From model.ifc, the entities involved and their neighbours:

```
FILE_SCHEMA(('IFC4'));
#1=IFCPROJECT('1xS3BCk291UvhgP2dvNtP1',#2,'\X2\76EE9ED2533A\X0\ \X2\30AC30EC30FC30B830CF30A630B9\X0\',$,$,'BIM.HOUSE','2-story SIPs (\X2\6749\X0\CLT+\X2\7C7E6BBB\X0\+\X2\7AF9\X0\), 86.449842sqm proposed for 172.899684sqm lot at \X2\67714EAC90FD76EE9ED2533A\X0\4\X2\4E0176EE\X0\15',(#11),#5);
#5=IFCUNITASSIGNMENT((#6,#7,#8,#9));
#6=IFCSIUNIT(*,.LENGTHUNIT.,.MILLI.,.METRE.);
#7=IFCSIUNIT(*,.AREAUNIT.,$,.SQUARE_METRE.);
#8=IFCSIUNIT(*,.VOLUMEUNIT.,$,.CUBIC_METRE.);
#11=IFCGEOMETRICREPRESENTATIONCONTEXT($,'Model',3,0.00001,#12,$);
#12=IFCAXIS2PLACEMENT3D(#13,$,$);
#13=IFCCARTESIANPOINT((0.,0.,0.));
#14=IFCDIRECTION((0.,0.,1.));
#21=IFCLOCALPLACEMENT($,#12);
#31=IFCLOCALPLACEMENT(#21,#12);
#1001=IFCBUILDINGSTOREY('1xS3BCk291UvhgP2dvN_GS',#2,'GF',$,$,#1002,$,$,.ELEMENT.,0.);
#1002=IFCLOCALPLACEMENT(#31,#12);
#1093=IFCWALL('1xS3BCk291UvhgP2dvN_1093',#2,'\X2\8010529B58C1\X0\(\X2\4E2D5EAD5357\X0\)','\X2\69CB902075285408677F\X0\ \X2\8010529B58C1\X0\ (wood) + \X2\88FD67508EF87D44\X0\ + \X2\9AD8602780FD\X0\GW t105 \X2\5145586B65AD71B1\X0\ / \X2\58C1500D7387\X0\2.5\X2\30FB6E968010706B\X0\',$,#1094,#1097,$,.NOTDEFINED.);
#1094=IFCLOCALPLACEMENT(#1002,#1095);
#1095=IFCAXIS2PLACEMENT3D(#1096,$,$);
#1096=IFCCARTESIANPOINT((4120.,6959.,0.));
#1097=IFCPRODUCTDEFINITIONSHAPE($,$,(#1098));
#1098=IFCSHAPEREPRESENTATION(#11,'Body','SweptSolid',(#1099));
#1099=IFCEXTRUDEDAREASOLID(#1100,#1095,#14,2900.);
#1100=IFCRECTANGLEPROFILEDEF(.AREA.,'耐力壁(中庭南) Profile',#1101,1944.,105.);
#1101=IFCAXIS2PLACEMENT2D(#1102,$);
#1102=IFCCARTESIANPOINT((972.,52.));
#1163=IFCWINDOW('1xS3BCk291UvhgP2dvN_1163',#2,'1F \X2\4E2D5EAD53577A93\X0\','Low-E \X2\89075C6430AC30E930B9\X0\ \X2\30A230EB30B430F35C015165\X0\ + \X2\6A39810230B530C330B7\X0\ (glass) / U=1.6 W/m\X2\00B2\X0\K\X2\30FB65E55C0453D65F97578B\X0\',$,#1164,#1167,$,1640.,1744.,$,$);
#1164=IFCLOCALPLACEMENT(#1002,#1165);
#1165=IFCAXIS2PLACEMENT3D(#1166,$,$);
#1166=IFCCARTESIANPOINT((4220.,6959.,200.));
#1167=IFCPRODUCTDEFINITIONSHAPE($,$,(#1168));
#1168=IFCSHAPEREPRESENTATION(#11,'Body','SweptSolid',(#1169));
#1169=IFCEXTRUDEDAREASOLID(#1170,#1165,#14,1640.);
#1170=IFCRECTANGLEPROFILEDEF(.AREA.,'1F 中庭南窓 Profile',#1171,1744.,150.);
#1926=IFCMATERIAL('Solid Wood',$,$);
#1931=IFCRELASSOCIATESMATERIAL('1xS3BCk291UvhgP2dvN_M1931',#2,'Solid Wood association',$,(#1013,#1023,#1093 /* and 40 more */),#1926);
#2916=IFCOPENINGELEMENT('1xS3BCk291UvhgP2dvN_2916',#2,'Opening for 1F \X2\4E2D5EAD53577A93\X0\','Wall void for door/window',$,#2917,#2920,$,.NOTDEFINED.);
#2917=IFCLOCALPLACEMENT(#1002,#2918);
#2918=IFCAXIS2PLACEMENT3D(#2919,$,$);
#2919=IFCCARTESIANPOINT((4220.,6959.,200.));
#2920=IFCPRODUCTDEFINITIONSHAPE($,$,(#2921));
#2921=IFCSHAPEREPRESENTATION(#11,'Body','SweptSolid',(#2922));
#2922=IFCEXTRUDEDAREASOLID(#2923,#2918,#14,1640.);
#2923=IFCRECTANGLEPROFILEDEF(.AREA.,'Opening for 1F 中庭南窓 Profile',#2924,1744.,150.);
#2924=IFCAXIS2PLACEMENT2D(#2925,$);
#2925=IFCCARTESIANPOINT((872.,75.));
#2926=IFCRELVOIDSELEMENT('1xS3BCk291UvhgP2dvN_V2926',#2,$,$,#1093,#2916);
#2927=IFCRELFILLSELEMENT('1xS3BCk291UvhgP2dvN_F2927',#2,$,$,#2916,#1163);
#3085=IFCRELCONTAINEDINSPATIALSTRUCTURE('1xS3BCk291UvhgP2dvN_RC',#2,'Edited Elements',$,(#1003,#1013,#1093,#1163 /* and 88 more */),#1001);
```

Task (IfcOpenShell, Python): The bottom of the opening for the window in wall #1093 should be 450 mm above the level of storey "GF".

```python
import numpy as np
import ifcopenshell
import ifcopenshell.api.geometry
import ifcopenshell.geom
import ifcopenshell.util.element
import ifcopenshell.util.placement
import ifcopenshell.util.shape
import ifcopenshell.util.unit

model = ifcopenshell.open("model.ifc")
unit_scale = ifcopenshell.util.unit.calculate_unit_scale(model)

window = model.by_id(1163)
opening = window.FillsVoids[0].RelatingOpeningElement
storey = ifcopenshell.util.element.get_container(window, ifc_class="IfcBuildingStorey")
level = ifcopenshell.util.placement.get_local_placement(storey.ObjectPlacement)[2, 3]

# The opening's origin need not be at the sill, so measure its lowest point.
shape = ifcopenshell.geom.create_shape(ifcopenshell.geom.settings(), opening)
bottom = ifcopenshell.util.shape.get_shape_bottom_elevation(shape, shape.geometry) / unit_scale
dz = level + 0.45 / unit_scale - bottom

shift = np.array([0.0, 0.0, dz])
# The window is not placed relative to its opening, so move both.
for product in (opening, window):
    matrix = ifcopenshell.util.placement.get_local_placement(product.ObjectPlacement)
    matrix[:3, 3] += shift
    ifcopenshell.api.geometry.edit_object_placement(model, product=product, matrix=matrix, is_si=False)

print(f"moved by {dz * unit_scale:+.3f} m")

model.write("model-out.ifc")
```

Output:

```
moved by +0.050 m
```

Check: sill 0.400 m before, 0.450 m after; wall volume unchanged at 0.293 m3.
